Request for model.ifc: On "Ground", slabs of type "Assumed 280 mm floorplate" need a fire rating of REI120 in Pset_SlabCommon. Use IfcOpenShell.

First a look at what the model holds.

```python
import ifcopenshell
import ifcopenshell.util.element

model = ifcopenshell.open("model.ifc")
print(model.schema)
storey = next(s for s in model.by_type("IfcBuildingStorey") if s.Name == "Ground")
slabs = [e for e in ifcopenshell.util.element.get_decomposition(storey) if e.is_a("IfcSlab")]
seen = {}
for e in slabs:
    element_type = ifcopenshell.util.element.get_type(e)
    key = (element_type.Name if element_type != e and element_type else None, ifcopenshell.util.element.get_pset(e, "Pset_SlabCommon", "FireRating"))
    seen[key] = seen.get(key, 0) + 1
for (name, value), count in sorted(seen.items(), key=str):
    print(count, "x", name, "|", value)
```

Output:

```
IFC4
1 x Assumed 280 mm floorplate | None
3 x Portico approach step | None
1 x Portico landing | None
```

```python
import ifcopenshell
import ifcopenshell.api.pset
import ifcopenshell.util.element

model = ifcopenshell.open("model.ifc")

storey = next(s for s in model.by_type("IfcBuildingStorey") if s.Name == "Ground")
slabs = [e for e in ifcopenshell.util.element.get_decomposition(storey) if e.is_a("IfcSlab")]

count = 0
for e in slabs:
    element_type = ifcopenshell.util.element.get_type(e)
    if element_type in (None, e) or element_type.Name != "Assumed 280 mm floorplate":
        continue
    # add_pset returns the element's existing set when there is one.
    pset = ifcopenshell.api.pset.add_pset(model, product=e, name="Pset_SlabCommon")
    ifcopenshell.api.pset.edit_pset(model, pset=pset, properties={"FireRating": "REI120"})
    count += 1

print(count, "slabs updated")

model.write("model_v2.ifc")
```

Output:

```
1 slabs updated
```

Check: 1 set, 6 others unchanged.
